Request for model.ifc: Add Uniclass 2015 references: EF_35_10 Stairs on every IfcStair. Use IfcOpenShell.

First a look at what the model holds.

```python
import ifcopenshell

model = ifcopenshell.open("model.ifc")
print(model.schema)
print("classifications:", [c.Name for c in model.by_type("IfcClassification")])
for ifc_class in ("IfcDoor", "IfcRoof", "IfcStair", "IfcWall", "IfcWindow"):
    print(ifc_class, len(model.by_type(ifc_class)))
```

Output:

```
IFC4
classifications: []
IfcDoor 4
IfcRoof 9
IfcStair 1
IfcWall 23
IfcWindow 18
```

```python
import ifcopenshell
import ifcopenshell.api.classification

model = ifcopenshell.open("model.ifc")

system = ifcopenshell.api.classification.add_classification(model, classification="Uniclass 2015")

codes = {
    "IfcStair": ("EF_35_10", "Stairs"),
}
for ifc_class, (code, name) in codes.items():
    products = model.by_type(ifc_class)
    ifcopenshell.api.classification.add_reference(
        model, products=products, classification=system, identification=code, name=name
    )
    print(code, len(products))

model.write("model_rev.ifc")
```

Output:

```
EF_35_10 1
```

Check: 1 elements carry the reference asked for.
